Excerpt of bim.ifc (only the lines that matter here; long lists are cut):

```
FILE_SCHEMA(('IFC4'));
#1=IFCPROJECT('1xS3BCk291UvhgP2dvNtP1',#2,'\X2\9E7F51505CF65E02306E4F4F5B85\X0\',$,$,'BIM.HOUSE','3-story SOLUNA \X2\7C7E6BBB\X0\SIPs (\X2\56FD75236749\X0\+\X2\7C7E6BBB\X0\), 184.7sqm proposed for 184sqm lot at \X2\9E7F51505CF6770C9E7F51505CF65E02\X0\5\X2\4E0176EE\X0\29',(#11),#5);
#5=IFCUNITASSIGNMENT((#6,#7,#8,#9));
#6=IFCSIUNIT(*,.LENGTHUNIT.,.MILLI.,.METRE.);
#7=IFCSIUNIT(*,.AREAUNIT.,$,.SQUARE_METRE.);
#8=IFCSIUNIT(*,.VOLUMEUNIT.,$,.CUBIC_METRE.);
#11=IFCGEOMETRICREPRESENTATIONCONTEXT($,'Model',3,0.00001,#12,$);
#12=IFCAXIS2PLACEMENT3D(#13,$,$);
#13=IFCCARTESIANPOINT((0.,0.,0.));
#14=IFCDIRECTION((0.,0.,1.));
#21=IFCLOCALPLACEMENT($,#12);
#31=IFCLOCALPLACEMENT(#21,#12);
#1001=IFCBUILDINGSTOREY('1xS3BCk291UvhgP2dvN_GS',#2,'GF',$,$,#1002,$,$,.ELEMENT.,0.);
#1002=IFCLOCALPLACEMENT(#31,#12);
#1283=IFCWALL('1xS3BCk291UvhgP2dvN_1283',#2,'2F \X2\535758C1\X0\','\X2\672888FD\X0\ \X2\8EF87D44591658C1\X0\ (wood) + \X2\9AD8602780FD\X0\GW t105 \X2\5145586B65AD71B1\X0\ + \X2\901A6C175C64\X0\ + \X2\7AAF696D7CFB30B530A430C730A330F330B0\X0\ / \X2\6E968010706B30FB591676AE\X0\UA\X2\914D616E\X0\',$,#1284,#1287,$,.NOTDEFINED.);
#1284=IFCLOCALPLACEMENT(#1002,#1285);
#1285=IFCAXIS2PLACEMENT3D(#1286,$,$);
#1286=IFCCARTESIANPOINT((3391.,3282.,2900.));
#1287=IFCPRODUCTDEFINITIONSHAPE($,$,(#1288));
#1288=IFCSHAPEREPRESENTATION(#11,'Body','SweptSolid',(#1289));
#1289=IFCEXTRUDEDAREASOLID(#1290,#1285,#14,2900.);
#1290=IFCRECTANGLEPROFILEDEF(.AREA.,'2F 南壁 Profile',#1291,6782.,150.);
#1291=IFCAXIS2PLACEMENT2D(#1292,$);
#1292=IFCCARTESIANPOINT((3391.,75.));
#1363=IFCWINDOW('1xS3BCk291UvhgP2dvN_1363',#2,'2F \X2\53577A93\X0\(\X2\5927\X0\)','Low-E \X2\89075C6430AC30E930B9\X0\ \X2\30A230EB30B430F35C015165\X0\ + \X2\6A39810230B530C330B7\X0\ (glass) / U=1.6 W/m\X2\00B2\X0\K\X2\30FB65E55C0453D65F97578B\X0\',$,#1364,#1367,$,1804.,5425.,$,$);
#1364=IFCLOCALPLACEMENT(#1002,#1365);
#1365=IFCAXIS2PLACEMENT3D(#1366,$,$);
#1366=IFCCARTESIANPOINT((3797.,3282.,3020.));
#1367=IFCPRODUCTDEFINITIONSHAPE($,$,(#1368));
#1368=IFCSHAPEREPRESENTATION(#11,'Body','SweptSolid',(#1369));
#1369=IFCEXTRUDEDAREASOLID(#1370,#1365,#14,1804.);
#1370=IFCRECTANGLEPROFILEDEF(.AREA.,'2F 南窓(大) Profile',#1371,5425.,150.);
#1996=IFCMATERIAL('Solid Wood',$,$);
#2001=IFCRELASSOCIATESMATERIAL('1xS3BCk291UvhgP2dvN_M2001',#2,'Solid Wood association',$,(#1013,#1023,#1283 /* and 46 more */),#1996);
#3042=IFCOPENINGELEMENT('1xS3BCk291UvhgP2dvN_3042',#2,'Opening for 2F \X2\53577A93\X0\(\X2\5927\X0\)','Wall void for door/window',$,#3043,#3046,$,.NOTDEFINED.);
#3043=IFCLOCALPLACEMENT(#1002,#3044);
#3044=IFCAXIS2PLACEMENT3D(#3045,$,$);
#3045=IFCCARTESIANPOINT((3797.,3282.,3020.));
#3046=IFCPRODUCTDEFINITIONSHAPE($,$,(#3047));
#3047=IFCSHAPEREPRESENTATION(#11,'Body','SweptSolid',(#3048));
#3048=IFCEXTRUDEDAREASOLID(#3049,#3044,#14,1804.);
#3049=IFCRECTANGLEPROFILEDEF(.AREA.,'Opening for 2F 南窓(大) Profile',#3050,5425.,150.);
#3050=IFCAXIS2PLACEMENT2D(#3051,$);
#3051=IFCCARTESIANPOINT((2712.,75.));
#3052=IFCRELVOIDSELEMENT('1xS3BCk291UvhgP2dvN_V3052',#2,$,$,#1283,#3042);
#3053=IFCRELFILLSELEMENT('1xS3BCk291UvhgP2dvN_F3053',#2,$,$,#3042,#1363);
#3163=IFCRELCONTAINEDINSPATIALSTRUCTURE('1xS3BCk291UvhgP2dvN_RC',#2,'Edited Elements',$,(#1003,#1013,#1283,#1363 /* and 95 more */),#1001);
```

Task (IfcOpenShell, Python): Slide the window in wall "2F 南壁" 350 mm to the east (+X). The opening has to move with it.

```python
import ifcopenshell
import ifcopenshell.api.geometry
import ifcopenshell.util.placement
import ifcopenshell.util.unit

model = ifcopenshell.open("bim.ifc")
unit_scale = ifcopenshell.util.unit.calculate_unit_scale(model)

window = model.by_id(1363)
opening = window.FillsVoids[0].RelatingOpeningElement
wall = opening.VoidsElements[0].RelatingBuildingElement

wall_matrix = ifcopenshell.util.placement.get_local_placement(wall.ObjectPlacement)
shift = wall_matrix[:3, 0] * 0.35 / unit_scale
before = ifcopenshell.util.placement.get_local_placement(window.ObjectPlacement)[:3, 3].copy()

# The window is not placed relative to its opening, so move both.
for product in (opening, window):
    matrix = ifcopenshell.util.placement.get_local_placement(product.ObjectPlacement)
    matrix[:3, 3] += shift
    ifcopenshell.api.geometry.edit_object_placement(model, product=product, matrix=matrix, is_si=False)

after = ifcopenshell.util.placement.get_local_placement(window.ObjectPlacement)[:3, 3]
print("window moved by", (after - before).round(3) + 0.0)

model.write("bim_v2.ifc")
```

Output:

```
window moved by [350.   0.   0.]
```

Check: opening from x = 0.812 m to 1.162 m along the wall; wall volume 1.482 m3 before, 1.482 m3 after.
